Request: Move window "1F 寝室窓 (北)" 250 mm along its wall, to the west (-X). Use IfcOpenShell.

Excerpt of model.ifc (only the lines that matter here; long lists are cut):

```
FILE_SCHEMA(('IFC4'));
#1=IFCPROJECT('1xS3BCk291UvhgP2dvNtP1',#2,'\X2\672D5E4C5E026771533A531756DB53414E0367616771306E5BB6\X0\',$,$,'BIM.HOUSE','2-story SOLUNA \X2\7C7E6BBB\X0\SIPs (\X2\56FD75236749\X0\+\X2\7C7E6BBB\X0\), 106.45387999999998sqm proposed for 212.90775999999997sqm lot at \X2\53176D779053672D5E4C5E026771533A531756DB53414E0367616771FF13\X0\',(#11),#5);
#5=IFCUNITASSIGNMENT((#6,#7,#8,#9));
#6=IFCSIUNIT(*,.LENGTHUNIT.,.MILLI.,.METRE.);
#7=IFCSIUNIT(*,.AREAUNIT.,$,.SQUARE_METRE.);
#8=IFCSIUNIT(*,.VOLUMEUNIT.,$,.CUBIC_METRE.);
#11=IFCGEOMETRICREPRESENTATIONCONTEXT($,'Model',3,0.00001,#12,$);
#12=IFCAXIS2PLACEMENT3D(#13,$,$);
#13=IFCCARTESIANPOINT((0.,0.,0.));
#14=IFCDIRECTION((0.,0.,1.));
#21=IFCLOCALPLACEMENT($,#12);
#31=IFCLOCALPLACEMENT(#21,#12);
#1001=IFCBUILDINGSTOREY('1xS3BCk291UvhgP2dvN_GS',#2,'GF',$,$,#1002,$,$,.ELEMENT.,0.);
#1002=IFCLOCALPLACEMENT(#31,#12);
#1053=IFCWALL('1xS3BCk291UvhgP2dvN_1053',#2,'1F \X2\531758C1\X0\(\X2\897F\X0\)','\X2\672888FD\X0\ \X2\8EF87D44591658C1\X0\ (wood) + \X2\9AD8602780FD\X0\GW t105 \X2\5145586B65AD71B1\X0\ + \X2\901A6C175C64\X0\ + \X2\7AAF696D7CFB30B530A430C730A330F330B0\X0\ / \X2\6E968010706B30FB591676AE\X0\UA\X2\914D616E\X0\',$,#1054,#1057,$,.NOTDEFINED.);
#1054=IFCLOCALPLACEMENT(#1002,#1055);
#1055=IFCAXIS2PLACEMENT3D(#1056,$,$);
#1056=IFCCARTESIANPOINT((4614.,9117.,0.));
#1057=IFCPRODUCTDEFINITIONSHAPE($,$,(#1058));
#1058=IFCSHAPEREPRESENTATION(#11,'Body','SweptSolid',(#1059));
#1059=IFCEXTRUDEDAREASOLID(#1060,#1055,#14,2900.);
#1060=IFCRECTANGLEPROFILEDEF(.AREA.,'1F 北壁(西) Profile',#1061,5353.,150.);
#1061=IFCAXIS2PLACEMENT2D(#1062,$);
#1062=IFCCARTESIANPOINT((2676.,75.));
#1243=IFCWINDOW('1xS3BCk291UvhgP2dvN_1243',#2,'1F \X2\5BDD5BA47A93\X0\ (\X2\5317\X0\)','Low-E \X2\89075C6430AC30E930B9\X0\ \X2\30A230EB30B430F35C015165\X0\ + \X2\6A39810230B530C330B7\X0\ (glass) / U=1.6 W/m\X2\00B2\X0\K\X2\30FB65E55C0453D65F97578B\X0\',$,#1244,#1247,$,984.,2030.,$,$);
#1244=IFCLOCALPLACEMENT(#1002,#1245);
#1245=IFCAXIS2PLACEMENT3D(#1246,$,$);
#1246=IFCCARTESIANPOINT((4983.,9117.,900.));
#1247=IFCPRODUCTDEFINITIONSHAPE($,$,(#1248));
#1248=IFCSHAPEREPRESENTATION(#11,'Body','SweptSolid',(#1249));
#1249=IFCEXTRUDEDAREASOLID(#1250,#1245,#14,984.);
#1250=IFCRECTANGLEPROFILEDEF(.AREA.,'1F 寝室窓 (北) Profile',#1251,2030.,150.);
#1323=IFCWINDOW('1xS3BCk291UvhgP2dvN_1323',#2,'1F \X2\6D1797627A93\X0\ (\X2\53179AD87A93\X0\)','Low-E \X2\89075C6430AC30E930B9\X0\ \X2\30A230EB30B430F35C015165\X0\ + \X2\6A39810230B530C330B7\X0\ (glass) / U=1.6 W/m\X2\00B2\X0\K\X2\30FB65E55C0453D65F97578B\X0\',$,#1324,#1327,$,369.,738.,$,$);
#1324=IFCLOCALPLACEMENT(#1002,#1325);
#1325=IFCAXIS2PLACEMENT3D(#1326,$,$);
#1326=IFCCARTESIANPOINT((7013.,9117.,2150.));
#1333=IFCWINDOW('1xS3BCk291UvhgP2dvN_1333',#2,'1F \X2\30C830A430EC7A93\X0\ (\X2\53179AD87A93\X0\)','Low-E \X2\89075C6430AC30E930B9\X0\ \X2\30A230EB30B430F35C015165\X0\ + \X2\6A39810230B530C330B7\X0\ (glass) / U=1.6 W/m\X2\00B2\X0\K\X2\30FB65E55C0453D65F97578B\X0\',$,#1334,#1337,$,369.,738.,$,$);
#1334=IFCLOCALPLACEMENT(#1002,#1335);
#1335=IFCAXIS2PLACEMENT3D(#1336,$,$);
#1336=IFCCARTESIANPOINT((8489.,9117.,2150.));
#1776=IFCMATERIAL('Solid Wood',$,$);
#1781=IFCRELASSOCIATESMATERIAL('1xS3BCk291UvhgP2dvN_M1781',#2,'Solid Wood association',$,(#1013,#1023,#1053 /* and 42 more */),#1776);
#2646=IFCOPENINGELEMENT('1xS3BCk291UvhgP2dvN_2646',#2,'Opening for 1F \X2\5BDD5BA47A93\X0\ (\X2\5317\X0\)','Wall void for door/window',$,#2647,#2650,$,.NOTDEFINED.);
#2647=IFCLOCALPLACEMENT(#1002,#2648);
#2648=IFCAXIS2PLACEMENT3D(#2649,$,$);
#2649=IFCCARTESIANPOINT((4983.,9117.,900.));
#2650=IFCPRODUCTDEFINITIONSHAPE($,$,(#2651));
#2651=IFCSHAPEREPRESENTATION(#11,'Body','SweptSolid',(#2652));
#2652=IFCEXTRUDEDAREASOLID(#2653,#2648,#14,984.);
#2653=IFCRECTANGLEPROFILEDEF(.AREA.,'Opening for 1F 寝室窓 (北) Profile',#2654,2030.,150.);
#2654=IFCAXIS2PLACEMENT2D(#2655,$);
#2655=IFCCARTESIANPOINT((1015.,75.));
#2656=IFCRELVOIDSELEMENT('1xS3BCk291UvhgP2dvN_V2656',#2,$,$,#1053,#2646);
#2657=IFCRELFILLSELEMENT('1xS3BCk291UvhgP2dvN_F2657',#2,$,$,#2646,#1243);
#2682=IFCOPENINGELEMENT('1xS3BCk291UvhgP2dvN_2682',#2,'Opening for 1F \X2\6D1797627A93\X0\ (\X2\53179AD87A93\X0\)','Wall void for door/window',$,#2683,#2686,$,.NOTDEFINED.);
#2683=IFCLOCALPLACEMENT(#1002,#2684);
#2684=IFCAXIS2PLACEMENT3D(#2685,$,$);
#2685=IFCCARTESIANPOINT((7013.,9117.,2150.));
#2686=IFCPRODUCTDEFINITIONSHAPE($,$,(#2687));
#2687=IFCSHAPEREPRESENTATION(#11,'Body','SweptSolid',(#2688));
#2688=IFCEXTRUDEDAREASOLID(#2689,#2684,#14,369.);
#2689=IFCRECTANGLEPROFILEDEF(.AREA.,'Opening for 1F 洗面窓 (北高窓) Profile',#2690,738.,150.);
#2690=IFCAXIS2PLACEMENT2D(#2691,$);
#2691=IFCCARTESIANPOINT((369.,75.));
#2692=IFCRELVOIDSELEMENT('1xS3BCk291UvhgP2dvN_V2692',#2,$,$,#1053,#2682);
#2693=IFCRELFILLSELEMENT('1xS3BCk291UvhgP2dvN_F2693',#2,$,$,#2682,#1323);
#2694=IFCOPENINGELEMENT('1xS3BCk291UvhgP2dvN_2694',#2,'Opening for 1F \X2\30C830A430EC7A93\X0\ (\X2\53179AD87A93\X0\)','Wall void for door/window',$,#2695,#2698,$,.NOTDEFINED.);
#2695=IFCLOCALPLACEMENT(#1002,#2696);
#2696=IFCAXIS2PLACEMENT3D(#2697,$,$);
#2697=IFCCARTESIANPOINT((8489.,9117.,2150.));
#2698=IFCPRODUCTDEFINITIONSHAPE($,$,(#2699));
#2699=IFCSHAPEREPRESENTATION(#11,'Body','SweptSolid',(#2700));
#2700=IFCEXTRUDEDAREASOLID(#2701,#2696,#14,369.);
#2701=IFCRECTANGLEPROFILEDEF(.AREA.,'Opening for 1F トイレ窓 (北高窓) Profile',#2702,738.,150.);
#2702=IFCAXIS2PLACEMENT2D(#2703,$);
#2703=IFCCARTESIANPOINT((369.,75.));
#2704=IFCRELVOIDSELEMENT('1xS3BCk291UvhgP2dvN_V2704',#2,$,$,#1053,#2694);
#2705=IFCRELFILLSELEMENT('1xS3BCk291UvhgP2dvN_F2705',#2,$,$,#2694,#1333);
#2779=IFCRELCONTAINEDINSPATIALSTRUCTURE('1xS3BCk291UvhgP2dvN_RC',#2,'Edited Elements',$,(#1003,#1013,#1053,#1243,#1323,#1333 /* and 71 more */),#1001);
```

```python
import ifcopenshell
import ifcopenshell.api.geometry
import ifcopenshell.util.placement
import ifcopenshell.util.unit

model = ifcopenshell.open("model.ifc")
unit_scale = ifcopenshell.util.unit.calculate_unit_scale(model)

window = model.by_guid("1xS3BCk291UvhgP2dvN_1243")
opening = window.FillsVoids[0].RelatingOpeningElement
wall = opening.VoidsElements[0].RelatingBuildingElement

wall_matrix = ifcopenshell.util.placement.get_local_placement(wall.ObjectPlacement)
shift = wall_matrix[:3, 0] * -0.25 / unit_scale
before = ifcopenshell.util.placement.get_local_placement(window.ObjectPlacement)[:3, 3].copy()

# The window is not placed relative to its opening, so move both.
for product in (opening, window):
    matrix = ifcopenshell.util.placement.get_local_placement(product.ObjectPlacement)
    matrix[:3, 3] += shift
    ifcopenshell.api.geometry.edit_object_placement(model, product=product, matrix=matrix, is_si=False)

after = ifcopenshell.util.placement.get_local_placement(window.ObjectPlacement)[:3, 3]
print("window moved by", (after - before).round(3) + 0.0)

model.write("model_updated.ifc")
```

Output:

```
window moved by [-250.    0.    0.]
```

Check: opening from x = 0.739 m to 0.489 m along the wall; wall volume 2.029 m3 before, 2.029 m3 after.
